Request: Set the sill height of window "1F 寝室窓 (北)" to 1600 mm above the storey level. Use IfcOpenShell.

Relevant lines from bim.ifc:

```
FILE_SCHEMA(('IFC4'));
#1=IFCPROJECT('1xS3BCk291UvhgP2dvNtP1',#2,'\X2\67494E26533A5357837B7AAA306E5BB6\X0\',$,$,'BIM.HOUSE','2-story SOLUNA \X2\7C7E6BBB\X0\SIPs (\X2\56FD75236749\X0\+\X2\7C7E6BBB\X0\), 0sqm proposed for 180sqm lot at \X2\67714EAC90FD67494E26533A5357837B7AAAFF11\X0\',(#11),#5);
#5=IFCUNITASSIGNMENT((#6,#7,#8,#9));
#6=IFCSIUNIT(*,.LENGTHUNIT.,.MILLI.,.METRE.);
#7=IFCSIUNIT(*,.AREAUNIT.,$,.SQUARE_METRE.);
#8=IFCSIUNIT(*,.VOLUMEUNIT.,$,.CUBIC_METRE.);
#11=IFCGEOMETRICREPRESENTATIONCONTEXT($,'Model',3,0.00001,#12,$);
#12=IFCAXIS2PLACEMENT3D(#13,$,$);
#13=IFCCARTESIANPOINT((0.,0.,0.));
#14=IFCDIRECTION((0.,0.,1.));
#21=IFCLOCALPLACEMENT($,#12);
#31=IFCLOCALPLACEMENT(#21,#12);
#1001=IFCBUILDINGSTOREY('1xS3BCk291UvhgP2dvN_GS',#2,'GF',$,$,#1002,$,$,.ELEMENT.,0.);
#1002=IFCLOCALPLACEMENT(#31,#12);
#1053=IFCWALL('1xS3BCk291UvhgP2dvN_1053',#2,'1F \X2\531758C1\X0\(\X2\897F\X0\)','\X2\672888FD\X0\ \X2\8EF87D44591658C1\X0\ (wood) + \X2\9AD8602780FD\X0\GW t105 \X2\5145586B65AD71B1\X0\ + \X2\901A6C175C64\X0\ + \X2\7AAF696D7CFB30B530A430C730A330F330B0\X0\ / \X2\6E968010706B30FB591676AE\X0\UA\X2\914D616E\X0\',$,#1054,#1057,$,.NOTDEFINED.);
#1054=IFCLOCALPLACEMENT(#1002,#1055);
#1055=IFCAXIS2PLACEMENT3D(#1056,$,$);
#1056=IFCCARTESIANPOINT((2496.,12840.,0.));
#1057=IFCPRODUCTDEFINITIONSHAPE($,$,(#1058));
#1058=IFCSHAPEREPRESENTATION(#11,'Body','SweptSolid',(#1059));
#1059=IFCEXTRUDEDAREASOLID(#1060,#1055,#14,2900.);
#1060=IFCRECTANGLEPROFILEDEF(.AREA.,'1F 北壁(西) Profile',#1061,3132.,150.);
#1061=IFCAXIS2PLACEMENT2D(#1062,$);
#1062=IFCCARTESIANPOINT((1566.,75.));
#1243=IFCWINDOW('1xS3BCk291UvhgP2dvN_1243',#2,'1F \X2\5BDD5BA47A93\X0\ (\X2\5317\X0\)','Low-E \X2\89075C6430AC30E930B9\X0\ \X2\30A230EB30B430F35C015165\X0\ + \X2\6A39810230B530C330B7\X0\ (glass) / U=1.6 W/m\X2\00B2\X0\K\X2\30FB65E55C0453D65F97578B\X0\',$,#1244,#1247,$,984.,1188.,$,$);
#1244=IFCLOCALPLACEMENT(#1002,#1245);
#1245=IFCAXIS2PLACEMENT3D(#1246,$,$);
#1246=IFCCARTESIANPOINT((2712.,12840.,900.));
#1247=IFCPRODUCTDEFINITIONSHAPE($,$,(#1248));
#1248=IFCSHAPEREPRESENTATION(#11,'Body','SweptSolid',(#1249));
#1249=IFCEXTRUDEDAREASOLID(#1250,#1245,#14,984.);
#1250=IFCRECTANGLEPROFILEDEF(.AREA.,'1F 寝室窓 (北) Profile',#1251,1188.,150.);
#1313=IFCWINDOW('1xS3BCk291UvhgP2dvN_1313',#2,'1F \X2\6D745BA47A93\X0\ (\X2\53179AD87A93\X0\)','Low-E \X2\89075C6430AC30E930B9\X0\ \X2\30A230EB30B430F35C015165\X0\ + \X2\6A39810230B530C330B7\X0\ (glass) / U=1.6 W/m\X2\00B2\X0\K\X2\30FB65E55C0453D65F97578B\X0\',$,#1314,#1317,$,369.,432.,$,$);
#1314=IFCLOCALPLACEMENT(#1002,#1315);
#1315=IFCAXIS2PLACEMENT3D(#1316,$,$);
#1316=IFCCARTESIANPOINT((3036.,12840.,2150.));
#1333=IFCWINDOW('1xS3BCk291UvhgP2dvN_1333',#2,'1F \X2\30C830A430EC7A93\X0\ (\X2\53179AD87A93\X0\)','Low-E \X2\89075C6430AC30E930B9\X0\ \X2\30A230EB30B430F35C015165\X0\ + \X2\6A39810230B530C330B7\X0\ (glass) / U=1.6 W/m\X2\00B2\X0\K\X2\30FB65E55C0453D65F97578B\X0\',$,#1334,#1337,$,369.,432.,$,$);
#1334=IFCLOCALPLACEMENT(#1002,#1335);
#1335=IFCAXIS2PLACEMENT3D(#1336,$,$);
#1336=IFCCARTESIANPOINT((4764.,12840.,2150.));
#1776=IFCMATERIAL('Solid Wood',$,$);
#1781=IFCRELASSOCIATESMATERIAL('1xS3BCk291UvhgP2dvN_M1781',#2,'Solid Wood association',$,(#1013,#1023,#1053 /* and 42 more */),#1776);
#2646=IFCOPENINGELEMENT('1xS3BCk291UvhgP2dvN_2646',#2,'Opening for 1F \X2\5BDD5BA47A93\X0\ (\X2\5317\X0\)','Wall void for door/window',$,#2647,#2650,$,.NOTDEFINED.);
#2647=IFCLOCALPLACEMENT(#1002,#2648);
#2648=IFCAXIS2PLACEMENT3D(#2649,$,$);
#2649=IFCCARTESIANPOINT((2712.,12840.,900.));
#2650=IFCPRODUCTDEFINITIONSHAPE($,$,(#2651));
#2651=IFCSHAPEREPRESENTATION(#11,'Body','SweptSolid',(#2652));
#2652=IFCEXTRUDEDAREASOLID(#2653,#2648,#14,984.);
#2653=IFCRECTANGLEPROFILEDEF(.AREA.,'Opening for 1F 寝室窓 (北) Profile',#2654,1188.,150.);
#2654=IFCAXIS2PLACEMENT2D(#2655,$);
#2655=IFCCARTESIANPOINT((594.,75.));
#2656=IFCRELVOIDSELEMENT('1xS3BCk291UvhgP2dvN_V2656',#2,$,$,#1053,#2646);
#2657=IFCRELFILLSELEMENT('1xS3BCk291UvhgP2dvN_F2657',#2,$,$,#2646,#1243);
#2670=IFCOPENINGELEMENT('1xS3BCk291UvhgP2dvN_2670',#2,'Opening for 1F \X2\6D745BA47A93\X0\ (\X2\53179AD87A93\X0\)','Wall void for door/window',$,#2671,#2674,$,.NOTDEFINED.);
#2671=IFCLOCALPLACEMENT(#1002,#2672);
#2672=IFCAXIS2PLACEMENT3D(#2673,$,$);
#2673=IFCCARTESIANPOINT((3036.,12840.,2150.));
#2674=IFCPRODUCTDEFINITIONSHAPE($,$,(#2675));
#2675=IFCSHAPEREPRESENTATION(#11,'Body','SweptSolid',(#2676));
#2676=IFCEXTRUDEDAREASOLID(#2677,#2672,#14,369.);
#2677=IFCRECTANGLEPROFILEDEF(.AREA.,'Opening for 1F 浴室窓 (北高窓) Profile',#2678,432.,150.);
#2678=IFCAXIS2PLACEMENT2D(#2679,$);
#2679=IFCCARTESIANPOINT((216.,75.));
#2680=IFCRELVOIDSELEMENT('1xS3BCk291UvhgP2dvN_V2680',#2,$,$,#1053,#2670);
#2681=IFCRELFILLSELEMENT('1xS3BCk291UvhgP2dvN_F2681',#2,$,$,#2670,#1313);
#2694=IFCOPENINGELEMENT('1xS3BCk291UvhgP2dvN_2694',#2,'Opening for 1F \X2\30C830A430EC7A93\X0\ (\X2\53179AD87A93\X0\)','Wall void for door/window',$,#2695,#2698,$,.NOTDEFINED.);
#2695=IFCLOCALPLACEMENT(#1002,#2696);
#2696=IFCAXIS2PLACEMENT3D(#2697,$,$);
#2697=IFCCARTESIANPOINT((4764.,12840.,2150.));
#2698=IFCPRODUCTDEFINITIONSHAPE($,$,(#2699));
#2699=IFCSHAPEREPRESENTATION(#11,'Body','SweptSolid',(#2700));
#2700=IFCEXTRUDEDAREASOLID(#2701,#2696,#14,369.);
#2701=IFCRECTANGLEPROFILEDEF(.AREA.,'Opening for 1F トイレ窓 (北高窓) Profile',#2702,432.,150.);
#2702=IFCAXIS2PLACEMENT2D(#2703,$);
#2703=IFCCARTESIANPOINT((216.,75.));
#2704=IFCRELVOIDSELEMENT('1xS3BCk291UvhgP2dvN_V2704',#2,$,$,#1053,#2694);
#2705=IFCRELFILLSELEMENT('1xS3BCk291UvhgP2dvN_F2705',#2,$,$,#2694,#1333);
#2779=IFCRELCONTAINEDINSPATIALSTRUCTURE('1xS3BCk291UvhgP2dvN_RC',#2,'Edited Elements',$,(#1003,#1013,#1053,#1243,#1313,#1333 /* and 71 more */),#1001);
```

```python
import numpy as np
import ifcopenshell
import ifcopenshell.api.geometry
import ifcopenshell.geom
import ifcopenshell.util.element
import ifcopenshell.util.placement
import ifcopenshell.util.shape
import ifcopenshell.util.unit

model = ifcopenshell.open("bim.ifc")
unit_scale = ifcopenshell.util.unit.calculate_unit_scale(model)

window = model.by_guid("1xS3BCk291UvhgP2dvN_1243")
opening = window.FillsVoids[0].RelatingOpeningElement
storey = ifcopenshell.util.element.get_container(window, ifc_class="IfcBuildingStorey")
level = ifcopenshell.util.placement.get_local_placement(storey.ObjectPlacement)[2, 3]

# The opening's origin need not be at the sill, so measure its lowest point.
shape = ifcopenshell.geom.create_shape(ifcopenshell.geom.settings(), opening)
bottom = ifcopenshell.util.shape.get_shape_bottom_elevation(shape, shape.geometry) / unit_scale
dz = level + 1.6 / unit_scale - bottom

shift = np.array([0.0, 0.0, dz])
# The window is not placed relative to its opening, so move both.
for product in (opening, window):
    matrix = ifcopenshell.util.placement.get_local_placement(product.ObjectPlacement)
    matrix[:3, 3] += shift
    ifcopenshell.api.geometry.edit_object_placement(model, product=product, matrix=matrix, is_si=False)

print(f"moved by {dz * unit_scale:+.3f} m")

model.write("bim_rev.ifc")
```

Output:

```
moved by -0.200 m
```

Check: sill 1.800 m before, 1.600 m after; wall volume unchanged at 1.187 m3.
